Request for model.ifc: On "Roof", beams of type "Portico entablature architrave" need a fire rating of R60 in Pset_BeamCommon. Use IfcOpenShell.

First a look at what the model holds.

```python
import ifcopenshell
import ifcopenshell.util.element

model = ifcopenshell.open("model.ifc")
print(model.schema)
storey = next(s for s in model.by_type("IfcBuildingStorey") if s.Name == "Roof")
beams = [e for e in ifcopenshell.util.element.get_decomposition(storey) if e.is_a("IfcBeam")]
seen = {}
for e in beams:
    element_type = ifcopenshell.util.element.get_type(e)
    key = (element_type.Name if element_type != e and element_type else None, ifcopenshell.util.element.get_pset(e, "Pset_BeamCommon", "FireRating"))
    seen[key] = seen.get(key, 0) + 1
for (name, value), count in sorted(seen.items(), key=str):
    print(count, "x", name, "|", value)
```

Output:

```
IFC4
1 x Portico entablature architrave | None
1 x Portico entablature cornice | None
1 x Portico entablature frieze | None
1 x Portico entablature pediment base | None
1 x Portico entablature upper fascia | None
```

```python
import ifcopenshell
import ifcopenshell.api.pset
import ifcopenshell.util.element

model = ifcopenshell.open("model.ifc")

storey = next(s for s in model.by_type("IfcBuildingStorey") if s.Name == "Roof")
beams = [e for e in ifcopenshell.util.element.get_decomposition(storey) if e.is_a("IfcBeam")]

count = 0
for e in beams:
    element_type = ifcopenshell.util.element.get_type(e)
    if element_type in (None, e) or element_type.Name != "Portico entablature architrave":
        continue
    # add_pset returns the element's existing set when there is one.
    pset = ifcopenshell.api.pset.add_pset(model, product=e, name="Pset_BeamCommon")
    ifcopenshell.api.pset.edit_pset(model, pset=pset, properties={"FireRating": "R60"})
    count += 1

print(count, "beams updated")

model.write("model_edited.ifc")
```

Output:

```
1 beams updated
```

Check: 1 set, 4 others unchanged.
